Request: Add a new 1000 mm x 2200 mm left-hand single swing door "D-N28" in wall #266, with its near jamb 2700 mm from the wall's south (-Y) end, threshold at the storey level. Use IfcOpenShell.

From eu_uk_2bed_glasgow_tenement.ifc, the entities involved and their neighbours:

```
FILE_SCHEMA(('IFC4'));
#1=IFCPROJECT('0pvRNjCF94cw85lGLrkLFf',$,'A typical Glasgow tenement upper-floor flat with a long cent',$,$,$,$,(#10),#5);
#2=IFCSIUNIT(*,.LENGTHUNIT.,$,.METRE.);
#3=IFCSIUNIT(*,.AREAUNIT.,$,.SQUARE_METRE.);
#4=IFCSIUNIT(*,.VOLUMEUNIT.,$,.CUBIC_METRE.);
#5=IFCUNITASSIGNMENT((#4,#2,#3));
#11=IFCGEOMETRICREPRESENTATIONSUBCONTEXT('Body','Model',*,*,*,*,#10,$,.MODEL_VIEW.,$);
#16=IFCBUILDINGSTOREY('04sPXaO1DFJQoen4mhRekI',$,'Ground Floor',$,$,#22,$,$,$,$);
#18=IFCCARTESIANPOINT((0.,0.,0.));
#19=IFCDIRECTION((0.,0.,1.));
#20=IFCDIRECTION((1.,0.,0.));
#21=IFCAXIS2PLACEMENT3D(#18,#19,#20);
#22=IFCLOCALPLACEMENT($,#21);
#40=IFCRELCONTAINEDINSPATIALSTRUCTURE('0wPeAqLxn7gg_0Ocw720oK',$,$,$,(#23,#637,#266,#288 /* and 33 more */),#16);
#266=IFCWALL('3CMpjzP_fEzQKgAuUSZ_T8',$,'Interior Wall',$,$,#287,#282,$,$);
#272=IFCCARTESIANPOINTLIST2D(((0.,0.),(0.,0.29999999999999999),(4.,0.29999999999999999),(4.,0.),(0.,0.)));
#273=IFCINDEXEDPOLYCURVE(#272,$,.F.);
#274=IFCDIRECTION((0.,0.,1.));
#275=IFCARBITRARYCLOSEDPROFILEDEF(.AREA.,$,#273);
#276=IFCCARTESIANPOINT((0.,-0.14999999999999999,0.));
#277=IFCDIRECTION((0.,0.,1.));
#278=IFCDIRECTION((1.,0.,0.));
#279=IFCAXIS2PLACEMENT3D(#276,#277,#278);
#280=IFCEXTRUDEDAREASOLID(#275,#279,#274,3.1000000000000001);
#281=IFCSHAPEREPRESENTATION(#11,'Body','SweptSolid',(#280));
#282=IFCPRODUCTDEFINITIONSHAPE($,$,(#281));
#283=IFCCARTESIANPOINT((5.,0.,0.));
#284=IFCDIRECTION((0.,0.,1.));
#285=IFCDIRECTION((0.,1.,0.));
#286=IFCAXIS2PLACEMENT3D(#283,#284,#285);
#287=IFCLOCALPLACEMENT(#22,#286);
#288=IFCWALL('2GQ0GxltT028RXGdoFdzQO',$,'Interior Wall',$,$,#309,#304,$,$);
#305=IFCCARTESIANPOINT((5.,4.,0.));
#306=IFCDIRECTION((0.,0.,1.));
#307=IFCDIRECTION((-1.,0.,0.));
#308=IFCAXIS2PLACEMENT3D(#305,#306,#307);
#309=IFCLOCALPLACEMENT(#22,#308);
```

```python
import numpy as np
import ifcopenshell
import ifcopenshell.api.feature
import ifcopenshell.api.geometry
import ifcopenshell.api.root
import ifcopenshell.api.spatial
import ifcopenshell.geom
import ifcopenshell.util.element
import ifcopenshell.util.placement
import ifcopenshell.util.representation
import ifcopenshell.util.shape
import ifcopenshell.util.unit

model = ifcopenshell.open("eu_uk_2bed_glasgow_tenement.ifc")
unit_scale = ifcopenshell.util.unit.calculate_unit_scale(model)
settings = ifcopenshell.geom.settings()


def volume(element):
    """Net volume in cubic metres, openings subtracted."""
    shape = ifcopenshell.geom.create_shape(settings, element)
    return ifcopenshell.util.shape.get_volume(shape.geometry)


wall = model.by_guid("3CMpjzP_fEzQKgAuUSZ_T8")
storey = ifcopenshell.util.element.get_container(wall, ifc_class="IfcBuildingStorey")
context = ifcopenshell.util.representation.get_context(model, "Model", "Body", "MODEL_VIEW")
before = volume(wall)

width, height, from_end, sill = 1, 2.2, 2.7, 0.0  # metres

# The wall runs along its own X axis, and the end named is its -X end.
wall_shape = ifcopenshell.geom.create_shape(settings, wall)
x, y, z = ifcopenshell.util.shape.get_vertices(wall_shape.geometry).T
start = x.min() + from_end
face, thickness = float(y.min()), float(y.max() - y.min())
wall_matrix = ifcopenshell.util.placement.get_local_placement(wall.ObjectPlacement)
level = ifcopenshell.util.placement.get_local_placement(storey.ObjectPlacement)[2, 3]


def in_wall(x, y):
    """Placement at x, y metres in the wall's axes, at sill height."""
    matrix = wall_matrix.copy()
    matrix[:, 3] = wall_matrix @ np.array([x / unit_scale, y / unit_scale, 0.0, 1.0])
    matrix[2, 3] = level + sill / unit_scale
    return matrix


# Opening: a box that overshoots both wall faces by 50 mm.
opening = ifcopenshell.api.root.create_entity(model, ifc_class="IfcOpeningElement", predefined_type="OPENING")
box = ifcopenshell.api.geometry.add_wall_representation(
    model, context=context, length=width, height=height, thickness=thickness + 0.1
)
ifcopenshell.api.geometry.assign_representation(model, product=opening, representation=box)
ifcopenshell.api.geometry.edit_object_placement(model, product=opening, matrix=in_wall(start, face - 0.05), is_si=False)
ifcopenshell.api.feature.add_feature(model, feature=opening, element=wall)

door = ifcopenshell.api.root.create_entity(model, ifc_class="IfcDoor", name="D-N28", predefined_type="DOOR")
door.OverallWidth, door.OverallHeight = width / unit_scale, height / unit_scale
door.OperationType = "SINGLE_SWING_LEFT"
body = ifcopenshell.api.geometry.add_door_representation(
    model,
    context=context,
    overall_width=door.OverallWidth,
    overall_height=door.OverallHeight,
    operation_type="SINGLE_SWING_LEFT",
    lining_properties={"LiningDepth": thickness / unit_scale, "ThresholdDepth": thickness / unit_scale},
)
ifcopenshell.api.geometry.assign_representation(model, product=door, representation=body)
ifcopenshell.api.spatial.assign_container(model, products=[door], relating_structure=storey)
ifcopenshell.api.feature.add_filling(model, opening=opening, element=door)

# The lining spans the wall, so the door starts at the wall face.
ifcopenshell.api.geometry.edit_object_placement(model, product=door, matrix=in_wall(start, face), is_si=False)

after = volume(wall)

print(f"wall volume {before:.3f} -> {after:.3f} m3")

model.write("eu_uk_2bed_glasgow_tenement_rev.ifc")
```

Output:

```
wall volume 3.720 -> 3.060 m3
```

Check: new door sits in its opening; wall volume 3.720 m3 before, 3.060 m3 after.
